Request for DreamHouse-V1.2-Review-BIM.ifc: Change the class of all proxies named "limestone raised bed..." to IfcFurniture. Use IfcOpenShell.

First a look at what the model holds.

```python
import re

import ifcopenshell

model = ifcopenshell.open("DreamHouse-V1.2-Review-BIM.ifc")
print(model.schema)
seen = {}
for e in model.by_type("IfcBuildingElementProxy"):
    name = re.sub(r":\d+(:\d+)?$", "", e.Name or "")  # drop the element id that some exporters append
    seen[name] = seen.get(name, 0) + 1
for name, count in sorted(seen.items()):
    print(count, "x", name)
```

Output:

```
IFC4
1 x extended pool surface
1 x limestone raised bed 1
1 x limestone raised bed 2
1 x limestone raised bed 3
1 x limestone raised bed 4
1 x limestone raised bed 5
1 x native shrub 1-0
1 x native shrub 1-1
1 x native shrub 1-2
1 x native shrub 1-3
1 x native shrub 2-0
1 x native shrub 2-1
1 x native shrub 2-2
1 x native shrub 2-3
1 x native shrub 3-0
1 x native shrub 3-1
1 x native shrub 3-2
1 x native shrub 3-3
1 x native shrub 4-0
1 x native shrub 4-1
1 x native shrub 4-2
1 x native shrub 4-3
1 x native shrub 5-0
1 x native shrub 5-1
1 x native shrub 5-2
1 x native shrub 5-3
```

```python
import ifcopenshell
import ifcopenshell.api.root

model = ifcopenshell.open("DreamHouse-V1.2-Review-BIM.ifc")

proxies = [e.id() for e in model.by_type("IfcBuildingElementProxy") if (e.Name or "").startswith("limestone raised bed")]
for step_id in proxies:
    proxy = model.by_id(step_id)
    ifcopenshell.api.root.reassign_class(model, product=proxy, ifc_class="IfcFurniture")

print(sum(model.by_id(i).is_a("IfcFurniture") for i in proxies), "reclassified")

model.write("DreamHouse-V1.2-Review-BIM_rev.ifc")
```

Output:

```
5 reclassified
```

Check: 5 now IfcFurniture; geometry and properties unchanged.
